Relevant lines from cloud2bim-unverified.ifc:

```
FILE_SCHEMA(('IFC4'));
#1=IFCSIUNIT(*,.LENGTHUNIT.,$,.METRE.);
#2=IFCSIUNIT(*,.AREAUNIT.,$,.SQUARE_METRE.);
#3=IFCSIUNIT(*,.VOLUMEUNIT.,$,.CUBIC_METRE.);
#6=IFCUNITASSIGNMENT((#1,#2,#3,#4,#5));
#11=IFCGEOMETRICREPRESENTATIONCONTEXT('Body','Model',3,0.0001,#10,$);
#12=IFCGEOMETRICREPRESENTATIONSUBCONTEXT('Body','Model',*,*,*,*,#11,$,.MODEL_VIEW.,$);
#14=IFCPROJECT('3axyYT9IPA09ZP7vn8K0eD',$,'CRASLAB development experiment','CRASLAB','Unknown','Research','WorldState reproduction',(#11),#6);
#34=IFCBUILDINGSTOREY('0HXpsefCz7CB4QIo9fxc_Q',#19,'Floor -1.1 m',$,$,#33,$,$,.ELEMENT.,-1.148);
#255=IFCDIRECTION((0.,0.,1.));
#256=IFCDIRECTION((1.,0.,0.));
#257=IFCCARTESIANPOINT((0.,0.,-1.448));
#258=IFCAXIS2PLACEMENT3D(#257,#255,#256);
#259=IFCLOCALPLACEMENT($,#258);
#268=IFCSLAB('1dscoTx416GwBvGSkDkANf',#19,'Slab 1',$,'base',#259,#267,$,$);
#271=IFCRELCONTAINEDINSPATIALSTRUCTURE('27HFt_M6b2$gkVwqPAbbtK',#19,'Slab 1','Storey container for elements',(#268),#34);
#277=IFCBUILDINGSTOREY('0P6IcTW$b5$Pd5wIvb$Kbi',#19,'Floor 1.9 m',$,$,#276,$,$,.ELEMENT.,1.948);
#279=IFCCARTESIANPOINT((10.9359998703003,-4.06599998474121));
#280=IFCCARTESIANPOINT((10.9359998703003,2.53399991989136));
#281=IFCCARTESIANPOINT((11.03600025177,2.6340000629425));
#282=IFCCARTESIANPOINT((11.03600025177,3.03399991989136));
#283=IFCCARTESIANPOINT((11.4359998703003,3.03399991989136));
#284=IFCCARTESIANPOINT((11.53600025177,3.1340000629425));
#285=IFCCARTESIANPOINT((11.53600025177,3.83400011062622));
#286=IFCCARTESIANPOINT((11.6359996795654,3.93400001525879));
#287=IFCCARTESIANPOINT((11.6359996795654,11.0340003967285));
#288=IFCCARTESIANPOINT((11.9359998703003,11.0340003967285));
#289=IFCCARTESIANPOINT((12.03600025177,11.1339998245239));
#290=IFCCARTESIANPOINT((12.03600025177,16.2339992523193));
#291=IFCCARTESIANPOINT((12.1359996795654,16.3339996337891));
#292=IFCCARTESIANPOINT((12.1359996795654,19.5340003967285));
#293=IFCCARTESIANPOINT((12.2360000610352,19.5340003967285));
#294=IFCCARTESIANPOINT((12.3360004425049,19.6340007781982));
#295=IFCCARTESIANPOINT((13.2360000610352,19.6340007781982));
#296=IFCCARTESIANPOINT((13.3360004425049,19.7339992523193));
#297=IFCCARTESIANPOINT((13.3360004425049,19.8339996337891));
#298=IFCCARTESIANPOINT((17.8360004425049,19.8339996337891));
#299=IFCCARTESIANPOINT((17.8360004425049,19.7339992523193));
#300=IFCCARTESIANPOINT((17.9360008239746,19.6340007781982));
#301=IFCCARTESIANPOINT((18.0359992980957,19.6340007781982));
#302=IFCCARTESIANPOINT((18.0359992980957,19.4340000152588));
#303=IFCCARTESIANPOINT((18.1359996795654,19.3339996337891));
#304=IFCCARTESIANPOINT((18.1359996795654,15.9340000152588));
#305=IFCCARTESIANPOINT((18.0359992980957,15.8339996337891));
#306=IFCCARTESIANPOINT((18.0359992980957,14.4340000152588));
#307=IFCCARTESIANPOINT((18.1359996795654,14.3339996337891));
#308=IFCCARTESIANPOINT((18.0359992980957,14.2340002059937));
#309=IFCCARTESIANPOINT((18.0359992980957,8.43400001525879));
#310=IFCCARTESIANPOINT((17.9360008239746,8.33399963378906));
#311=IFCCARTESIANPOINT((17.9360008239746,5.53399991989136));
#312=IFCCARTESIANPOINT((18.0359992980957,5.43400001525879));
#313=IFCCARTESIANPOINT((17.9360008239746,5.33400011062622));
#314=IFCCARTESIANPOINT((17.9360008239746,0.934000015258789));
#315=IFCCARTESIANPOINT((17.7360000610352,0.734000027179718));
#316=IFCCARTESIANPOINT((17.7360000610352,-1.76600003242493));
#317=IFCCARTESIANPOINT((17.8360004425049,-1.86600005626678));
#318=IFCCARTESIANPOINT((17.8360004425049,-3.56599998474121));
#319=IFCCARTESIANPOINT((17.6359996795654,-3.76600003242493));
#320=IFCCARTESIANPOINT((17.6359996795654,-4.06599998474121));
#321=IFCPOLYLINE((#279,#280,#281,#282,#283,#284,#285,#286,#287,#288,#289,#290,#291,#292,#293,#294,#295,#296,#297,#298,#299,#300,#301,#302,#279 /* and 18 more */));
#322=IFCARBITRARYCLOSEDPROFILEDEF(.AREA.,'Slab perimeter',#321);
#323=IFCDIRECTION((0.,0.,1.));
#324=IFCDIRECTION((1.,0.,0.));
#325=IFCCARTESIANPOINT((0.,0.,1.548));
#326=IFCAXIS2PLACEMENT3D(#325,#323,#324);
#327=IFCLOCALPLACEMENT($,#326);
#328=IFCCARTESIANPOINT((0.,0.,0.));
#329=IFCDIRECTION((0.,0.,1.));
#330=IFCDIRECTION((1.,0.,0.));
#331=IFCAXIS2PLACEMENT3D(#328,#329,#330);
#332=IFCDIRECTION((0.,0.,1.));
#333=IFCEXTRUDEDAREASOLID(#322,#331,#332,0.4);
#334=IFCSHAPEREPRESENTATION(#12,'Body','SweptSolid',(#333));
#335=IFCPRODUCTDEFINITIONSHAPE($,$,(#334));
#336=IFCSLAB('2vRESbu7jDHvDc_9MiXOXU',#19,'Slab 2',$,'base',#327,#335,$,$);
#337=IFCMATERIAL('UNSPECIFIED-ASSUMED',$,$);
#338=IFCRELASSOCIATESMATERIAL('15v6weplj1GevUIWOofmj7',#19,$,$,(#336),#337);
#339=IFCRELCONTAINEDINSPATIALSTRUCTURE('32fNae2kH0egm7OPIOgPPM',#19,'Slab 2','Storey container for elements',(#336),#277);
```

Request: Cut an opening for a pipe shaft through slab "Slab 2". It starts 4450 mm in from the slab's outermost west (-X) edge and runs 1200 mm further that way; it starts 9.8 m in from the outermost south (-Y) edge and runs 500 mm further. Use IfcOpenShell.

```python
import numpy as np
import ifcopenshell
import ifcopenshell.api.feature
import ifcopenshell.api.geometry
import ifcopenshell.api.root
import ifcopenshell.geom
import ifcopenshell.util.placement
import ifcopenshell.util.representation
import ifcopenshell.util.shape
import ifcopenshell.util.unit

model = ifcopenshell.open("cloud2bim-unverified.ifc")
unit_scale = ifcopenshell.util.unit.calculate_unit_scale(model)
settings = ifcopenshell.geom.settings()


def volume(element):
    """Net volume in cubic metres, openings subtracted."""
    shape = ifcopenshell.geom.create_shape(settings, element)
    return ifcopenshell.util.shape.get_volume(shape.geometry)


slab = model.by_id(336)
before = volume(slab)

# Extent in the slab's own axes, in metres. The edges named are its -X and -Y sides.
slab_shape = ifcopenshell.geom.create_shape(settings, slab)
vertices = ifcopenshell.util.shape.get_vertices(slab_shape.geometry)
x_min, y_min, bottom = vertices.min(axis=0)
top = vertices[:, 2].max()

opening = ifcopenshell.api.root.create_entity(model, ifc_class="IfcOpeningElement", name="Pipe shaft opening", predefined_type="OPENING")
context = ifcopenshell.util.representation.get_context(model, "Model", "Body", "MODEL_VIEW")
width, depth = 1.2, 0.5
outline = [(0.0, 0.0), (width, 0.0), (width, depth), (0.0, depth), (0.0, 0.0)]
# Overshoot both faces by 50 mm so the cut is clean.
shape = ifcopenshell.api.geometry.add_slab_representation(
    model, context=context, depth=top - bottom + 0.1, polyline=outline
)
ifcopenshell.api.geometry.assign_representation(model, product=opening, representation=shape)

matrix = ifcopenshell.util.placement.get_local_placement(slab.ObjectPlacement)
matrix[:, 3] = matrix @ np.append(np.array([x_min + 4.45, y_min + 9.8, bottom - 0.05]) / unit_scale, 1.0)
ifcopenshell.api.geometry.edit_object_placement(model, product=opening, matrix=matrix, is_si=False)
ifcopenshell.api.feature.add_feature(model, feature=opening, element=slab)

after = volume(slab)

print(f"slab volume {before:.3f} -> {after:.3f} m3")

model.write("cloud2bim-unverified_edited.ifc")
```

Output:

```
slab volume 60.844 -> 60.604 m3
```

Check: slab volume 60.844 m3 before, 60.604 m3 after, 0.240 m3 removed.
